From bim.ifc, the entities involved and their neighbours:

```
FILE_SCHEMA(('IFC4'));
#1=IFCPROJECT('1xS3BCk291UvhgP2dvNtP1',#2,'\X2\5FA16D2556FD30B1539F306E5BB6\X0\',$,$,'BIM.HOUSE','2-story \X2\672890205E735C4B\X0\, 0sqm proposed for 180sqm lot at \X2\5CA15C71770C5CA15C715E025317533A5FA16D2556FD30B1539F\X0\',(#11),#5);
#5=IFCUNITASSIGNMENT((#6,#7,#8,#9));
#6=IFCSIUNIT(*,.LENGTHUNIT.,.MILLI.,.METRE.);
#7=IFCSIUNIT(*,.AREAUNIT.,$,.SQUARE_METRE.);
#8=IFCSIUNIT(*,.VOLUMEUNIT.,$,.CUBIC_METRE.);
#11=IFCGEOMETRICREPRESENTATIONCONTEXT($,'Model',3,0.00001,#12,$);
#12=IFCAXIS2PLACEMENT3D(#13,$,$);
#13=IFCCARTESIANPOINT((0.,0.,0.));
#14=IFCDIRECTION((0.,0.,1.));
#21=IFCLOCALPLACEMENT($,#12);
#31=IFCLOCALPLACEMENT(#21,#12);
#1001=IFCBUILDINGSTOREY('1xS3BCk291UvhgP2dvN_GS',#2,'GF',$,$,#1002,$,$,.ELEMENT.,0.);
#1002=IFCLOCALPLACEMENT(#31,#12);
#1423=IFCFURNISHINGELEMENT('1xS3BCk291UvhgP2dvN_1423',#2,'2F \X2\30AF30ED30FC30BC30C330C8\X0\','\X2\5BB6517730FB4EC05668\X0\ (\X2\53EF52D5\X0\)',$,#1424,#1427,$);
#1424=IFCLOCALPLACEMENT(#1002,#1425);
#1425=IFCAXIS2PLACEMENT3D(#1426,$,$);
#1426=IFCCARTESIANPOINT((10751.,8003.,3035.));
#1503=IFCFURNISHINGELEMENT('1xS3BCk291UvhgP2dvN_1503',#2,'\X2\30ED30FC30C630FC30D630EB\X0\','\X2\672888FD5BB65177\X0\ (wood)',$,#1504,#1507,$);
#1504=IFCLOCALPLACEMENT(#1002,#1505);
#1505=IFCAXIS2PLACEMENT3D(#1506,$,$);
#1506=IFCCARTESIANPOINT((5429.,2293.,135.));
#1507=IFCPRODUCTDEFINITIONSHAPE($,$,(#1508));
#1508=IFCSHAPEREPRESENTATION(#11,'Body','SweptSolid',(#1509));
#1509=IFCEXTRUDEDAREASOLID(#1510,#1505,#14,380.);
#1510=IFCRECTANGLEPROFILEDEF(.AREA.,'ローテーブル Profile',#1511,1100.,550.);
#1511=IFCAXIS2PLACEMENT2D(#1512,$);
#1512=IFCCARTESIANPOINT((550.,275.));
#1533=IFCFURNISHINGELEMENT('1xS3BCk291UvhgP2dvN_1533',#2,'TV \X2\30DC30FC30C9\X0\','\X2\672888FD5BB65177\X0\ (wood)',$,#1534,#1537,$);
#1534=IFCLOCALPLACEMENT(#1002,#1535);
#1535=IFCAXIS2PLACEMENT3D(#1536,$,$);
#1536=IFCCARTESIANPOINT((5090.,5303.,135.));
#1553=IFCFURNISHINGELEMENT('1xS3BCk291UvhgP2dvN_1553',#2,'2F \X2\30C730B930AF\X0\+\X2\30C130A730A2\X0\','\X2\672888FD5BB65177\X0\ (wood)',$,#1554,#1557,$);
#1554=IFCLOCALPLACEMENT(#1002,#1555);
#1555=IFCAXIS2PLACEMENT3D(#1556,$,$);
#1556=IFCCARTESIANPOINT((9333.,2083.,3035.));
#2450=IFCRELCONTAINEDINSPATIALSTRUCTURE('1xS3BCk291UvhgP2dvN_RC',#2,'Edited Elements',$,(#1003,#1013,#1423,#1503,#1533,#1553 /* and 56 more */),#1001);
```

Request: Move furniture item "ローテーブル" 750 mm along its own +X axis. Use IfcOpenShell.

```python
import ifcopenshell
import ifcopenshell.api.geometry
import ifcopenshell.util.placement
import ifcopenshell.util.unit

model = ifcopenshell.open("bim.ifc")
unit_scale = ifcopenshell.util.unit.calculate_unit_scale(model)

item = model.by_guid("1xS3BCk291UvhgP2dvN_1503")
matrix = ifcopenshell.util.placement.get_local_placement(item.ObjectPlacement)
matrix[:3, 3] += matrix[:3, 0] * 0.75 / unit_scale
ifcopenshell.api.geometry.edit_object_placement(model, product=item, matrix=matrix, is_si=False)

print(ifcopenshell.util.placement.get_local_placement(item.ObjectPlacement).round(3) + 0.0)

model.write("bim_v2.ifc")
```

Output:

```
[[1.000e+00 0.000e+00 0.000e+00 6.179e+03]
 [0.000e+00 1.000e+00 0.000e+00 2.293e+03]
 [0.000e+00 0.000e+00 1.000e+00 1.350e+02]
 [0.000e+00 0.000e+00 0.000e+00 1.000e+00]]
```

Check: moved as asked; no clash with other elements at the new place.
